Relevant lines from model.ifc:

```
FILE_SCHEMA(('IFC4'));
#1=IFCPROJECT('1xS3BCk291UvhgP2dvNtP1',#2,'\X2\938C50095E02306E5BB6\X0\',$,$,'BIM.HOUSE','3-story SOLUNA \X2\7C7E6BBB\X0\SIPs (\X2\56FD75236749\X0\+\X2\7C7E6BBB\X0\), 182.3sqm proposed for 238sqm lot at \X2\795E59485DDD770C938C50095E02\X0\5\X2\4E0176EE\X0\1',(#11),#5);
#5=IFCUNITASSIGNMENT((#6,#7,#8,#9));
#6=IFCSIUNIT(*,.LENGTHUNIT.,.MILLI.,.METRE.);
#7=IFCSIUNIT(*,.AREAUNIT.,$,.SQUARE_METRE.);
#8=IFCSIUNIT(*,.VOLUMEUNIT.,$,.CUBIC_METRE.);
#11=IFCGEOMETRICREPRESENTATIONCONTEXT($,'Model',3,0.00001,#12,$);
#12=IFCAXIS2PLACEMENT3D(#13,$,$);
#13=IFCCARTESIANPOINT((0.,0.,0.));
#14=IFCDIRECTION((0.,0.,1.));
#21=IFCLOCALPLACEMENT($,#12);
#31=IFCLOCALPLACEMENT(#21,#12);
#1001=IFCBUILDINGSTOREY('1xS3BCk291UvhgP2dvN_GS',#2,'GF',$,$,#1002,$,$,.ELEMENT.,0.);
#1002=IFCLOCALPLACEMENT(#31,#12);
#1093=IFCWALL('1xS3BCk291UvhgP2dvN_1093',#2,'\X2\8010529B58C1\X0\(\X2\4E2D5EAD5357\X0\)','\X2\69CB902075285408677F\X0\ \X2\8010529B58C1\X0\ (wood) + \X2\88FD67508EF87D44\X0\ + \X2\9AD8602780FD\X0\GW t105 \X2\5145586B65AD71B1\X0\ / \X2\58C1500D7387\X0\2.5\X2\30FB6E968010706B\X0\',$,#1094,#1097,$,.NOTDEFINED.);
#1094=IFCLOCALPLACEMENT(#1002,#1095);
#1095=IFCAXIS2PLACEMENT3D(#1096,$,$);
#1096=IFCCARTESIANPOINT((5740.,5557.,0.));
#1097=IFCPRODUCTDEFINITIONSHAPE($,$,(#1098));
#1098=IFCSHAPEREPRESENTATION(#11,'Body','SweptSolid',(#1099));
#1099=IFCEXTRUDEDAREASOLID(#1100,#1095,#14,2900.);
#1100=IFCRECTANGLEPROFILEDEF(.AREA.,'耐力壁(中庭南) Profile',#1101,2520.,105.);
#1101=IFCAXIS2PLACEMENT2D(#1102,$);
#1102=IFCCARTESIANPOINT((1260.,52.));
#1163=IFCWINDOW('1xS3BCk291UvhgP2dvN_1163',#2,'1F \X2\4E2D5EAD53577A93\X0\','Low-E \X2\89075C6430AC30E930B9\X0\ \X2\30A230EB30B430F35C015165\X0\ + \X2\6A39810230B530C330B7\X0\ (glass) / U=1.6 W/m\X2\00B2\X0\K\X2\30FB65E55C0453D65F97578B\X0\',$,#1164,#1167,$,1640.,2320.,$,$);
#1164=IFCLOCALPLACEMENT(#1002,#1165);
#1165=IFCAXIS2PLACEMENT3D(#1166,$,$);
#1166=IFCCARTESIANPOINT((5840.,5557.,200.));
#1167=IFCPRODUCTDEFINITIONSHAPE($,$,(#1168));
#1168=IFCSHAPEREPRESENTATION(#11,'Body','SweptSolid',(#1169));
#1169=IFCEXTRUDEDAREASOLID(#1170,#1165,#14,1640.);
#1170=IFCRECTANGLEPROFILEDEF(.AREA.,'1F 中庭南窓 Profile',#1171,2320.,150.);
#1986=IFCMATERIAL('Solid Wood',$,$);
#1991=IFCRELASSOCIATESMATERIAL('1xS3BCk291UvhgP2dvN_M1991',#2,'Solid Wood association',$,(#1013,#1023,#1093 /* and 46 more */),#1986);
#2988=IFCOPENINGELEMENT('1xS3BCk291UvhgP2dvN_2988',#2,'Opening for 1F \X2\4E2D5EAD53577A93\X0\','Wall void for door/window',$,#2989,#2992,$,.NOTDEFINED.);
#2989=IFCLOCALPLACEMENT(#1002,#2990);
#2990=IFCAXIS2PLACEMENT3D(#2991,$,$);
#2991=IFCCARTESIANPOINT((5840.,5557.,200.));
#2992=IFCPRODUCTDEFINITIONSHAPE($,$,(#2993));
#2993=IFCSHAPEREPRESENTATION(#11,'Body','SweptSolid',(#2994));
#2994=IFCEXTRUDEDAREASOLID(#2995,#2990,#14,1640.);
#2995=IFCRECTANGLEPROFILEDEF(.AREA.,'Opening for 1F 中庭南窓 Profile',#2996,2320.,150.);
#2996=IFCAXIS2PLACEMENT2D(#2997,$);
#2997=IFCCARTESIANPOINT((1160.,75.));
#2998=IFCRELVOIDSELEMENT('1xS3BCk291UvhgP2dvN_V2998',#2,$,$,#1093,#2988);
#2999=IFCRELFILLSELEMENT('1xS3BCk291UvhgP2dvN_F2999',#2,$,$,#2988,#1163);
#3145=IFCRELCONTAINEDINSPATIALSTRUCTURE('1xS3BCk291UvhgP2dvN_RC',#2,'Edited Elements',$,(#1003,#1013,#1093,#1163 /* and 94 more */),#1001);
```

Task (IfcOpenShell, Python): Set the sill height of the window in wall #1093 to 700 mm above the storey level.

```python
import numpy as np
import ifcopenshell
import ifcopenshell.api.geometry
import ifcopenshell.geom
import ifcopenshell.util.element
import ifcopenshell.util.placement
import ifcopenshell.util.shape
import ifcopenshell.util.unit

model = ifcopenshell.open("model.ifc")
unit_scale = ifcopenshell.util.unit.calculate_unit_scale(model)

window = model.by_guid("1xS3BCk291UvhgP2dvN_1163")
opening = window.FillsVoids[0].RelatingOpeningElement
storey = ifcopenshell.util.element.get_container(window, ifc_class="IfcBuildingStorey")
level = ifcopenshell.util.placement.get_local_placement(storey.ObjectPlacement)[2, 3]

# The opening's origin need not be at the sill, so measure its lowest point.
shape = ifcopenshell.geom.create_shape(ifcopenshell.geom.settings(), opening)
bottom = ifcopenshell.util.shape.get_shape_bottom_elevation(shape, shape.geometry) / unit_scale
dz = level + 700.0 - bottom

shift = np.array([0.0, 0.0, dz])
# The window is not placed relative to its opening, so move both.
for product in (opening, window):
    matrix = ifcopenshell.util.placement.get_local_placement(product.ObjectPlacement)
    matrix[:3, 3] += shift
    ifcopenshell.api.geometry.edit_object_placement(model, product=product, matrix=matrix, is_si=False)

print(f"moved by {dz * unit_scale:+.3f} m")

model.write("model_v2.ifc")
```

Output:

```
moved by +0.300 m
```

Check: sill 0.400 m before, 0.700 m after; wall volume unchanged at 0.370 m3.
